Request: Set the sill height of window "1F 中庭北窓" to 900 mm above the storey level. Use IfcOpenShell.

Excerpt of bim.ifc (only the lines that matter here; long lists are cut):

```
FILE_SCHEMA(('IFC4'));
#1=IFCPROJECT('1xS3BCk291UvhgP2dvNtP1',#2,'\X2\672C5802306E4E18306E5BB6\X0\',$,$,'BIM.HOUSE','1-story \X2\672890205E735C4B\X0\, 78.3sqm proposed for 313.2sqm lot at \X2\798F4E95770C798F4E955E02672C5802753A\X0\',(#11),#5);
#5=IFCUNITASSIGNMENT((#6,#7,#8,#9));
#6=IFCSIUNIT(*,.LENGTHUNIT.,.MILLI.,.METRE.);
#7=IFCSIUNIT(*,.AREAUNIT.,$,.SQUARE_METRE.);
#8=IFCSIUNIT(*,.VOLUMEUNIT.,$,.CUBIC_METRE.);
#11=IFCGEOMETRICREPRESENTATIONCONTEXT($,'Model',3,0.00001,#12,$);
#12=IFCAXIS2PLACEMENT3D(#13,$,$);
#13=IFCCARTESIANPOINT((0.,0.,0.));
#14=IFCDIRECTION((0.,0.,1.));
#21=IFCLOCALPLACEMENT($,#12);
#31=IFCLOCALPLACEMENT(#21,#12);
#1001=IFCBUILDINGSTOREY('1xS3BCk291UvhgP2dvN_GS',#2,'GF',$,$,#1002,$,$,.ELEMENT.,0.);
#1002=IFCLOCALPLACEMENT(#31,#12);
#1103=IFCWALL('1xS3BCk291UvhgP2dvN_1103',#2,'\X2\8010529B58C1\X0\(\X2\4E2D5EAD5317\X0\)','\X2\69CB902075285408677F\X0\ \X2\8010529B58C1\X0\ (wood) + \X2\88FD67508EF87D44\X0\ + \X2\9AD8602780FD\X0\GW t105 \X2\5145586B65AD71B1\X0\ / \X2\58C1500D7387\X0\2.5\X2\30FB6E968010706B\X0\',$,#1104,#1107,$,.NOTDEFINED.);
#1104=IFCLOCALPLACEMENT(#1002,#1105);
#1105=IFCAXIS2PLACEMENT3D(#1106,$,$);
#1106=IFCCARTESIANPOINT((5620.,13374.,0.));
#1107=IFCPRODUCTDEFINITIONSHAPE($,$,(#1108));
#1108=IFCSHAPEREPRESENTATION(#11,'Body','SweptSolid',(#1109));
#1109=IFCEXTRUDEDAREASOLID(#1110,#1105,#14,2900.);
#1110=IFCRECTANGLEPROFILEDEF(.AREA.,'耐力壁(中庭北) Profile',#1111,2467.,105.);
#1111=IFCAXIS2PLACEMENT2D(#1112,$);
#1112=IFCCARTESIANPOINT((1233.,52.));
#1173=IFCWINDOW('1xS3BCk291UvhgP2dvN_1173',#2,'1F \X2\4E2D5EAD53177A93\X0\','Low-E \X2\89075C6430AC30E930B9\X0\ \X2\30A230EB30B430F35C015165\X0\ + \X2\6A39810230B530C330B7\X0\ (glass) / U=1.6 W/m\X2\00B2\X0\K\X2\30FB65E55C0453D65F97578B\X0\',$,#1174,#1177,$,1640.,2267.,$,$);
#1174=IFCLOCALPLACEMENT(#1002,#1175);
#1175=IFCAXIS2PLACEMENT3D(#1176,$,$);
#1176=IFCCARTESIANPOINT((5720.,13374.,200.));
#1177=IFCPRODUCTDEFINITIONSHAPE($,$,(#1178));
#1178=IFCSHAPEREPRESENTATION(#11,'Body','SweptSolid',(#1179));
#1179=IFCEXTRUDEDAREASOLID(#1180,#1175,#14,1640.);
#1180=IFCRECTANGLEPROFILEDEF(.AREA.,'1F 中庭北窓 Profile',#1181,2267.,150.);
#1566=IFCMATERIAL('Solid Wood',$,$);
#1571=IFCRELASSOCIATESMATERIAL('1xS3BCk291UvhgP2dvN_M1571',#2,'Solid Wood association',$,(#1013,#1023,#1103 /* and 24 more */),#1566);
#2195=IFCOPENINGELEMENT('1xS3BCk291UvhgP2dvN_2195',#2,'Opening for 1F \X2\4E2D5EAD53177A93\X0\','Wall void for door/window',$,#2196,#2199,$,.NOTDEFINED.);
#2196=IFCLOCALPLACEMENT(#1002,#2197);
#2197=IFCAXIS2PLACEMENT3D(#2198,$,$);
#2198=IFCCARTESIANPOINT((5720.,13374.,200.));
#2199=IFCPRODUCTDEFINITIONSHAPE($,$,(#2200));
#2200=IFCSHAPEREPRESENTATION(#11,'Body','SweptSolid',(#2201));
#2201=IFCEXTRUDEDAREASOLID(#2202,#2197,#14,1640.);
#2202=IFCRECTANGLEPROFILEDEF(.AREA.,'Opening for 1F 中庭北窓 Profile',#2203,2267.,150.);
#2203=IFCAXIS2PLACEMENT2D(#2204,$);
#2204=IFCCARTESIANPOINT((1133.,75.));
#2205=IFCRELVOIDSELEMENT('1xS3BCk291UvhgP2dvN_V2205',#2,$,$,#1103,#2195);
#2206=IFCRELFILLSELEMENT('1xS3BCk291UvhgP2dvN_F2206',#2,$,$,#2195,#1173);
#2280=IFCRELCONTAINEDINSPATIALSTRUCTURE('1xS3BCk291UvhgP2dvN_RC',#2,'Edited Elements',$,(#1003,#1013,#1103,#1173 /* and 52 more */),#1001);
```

```python
import numpy as np
import ifcopenshell
import ifcopenshell.api.geometry
import ifcopenshell.geom
import ifcopenshell.util.element
import ifcopenshell.util.placement
import ifcopenshell.util.shape
import ifcopenshell.util.unit

model = ifcopenshell.open("bim.ifc")
unit_scale = ifcopenshell.util.unit.calculate_unit_scale(model)

window = model.by_guid("1xS3BCk291UvhgP2dvN_1173")
opening = window.FillsVoids[0].RelatingOpeningElement
storey = ifcopenshell.util.element.get_container(window, ifc_class="IfcBuildingStorey")
level = ifcopenshell.util.placement.get_local_placement(storey.ObjectPlacement)[2, 3]

# The opening's origin need not be at the sill, so measure its lowest point.
shape = ifcopenshell.geom.create_shape(ifcopenshell.geom.settings(), opening)
bottom = ifcopenshell.util.shape.get_shape_bottom_elevation(shape, shape.geometry) / unit_scale
dz = level + 900.0 - bottom

shift = np.array([0.0, 0.0, dz])
# The window is not placed relative to its opening, so move both.
for product in (opening, window):
    matrix = ifcopenshell.util.placement.get_local_placement(product.ObjectPlacement)
    matrix[:3, 3] += shift
    ifcopenshell.api.geometry.edit_object_placement(model, product=product, matrix=matrix, is_si=False)

print(f"moved by {dz * unit_scale:+.3f} m")

model.write("bim_updated.ifc")
```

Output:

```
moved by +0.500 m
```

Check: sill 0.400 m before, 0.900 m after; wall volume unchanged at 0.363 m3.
